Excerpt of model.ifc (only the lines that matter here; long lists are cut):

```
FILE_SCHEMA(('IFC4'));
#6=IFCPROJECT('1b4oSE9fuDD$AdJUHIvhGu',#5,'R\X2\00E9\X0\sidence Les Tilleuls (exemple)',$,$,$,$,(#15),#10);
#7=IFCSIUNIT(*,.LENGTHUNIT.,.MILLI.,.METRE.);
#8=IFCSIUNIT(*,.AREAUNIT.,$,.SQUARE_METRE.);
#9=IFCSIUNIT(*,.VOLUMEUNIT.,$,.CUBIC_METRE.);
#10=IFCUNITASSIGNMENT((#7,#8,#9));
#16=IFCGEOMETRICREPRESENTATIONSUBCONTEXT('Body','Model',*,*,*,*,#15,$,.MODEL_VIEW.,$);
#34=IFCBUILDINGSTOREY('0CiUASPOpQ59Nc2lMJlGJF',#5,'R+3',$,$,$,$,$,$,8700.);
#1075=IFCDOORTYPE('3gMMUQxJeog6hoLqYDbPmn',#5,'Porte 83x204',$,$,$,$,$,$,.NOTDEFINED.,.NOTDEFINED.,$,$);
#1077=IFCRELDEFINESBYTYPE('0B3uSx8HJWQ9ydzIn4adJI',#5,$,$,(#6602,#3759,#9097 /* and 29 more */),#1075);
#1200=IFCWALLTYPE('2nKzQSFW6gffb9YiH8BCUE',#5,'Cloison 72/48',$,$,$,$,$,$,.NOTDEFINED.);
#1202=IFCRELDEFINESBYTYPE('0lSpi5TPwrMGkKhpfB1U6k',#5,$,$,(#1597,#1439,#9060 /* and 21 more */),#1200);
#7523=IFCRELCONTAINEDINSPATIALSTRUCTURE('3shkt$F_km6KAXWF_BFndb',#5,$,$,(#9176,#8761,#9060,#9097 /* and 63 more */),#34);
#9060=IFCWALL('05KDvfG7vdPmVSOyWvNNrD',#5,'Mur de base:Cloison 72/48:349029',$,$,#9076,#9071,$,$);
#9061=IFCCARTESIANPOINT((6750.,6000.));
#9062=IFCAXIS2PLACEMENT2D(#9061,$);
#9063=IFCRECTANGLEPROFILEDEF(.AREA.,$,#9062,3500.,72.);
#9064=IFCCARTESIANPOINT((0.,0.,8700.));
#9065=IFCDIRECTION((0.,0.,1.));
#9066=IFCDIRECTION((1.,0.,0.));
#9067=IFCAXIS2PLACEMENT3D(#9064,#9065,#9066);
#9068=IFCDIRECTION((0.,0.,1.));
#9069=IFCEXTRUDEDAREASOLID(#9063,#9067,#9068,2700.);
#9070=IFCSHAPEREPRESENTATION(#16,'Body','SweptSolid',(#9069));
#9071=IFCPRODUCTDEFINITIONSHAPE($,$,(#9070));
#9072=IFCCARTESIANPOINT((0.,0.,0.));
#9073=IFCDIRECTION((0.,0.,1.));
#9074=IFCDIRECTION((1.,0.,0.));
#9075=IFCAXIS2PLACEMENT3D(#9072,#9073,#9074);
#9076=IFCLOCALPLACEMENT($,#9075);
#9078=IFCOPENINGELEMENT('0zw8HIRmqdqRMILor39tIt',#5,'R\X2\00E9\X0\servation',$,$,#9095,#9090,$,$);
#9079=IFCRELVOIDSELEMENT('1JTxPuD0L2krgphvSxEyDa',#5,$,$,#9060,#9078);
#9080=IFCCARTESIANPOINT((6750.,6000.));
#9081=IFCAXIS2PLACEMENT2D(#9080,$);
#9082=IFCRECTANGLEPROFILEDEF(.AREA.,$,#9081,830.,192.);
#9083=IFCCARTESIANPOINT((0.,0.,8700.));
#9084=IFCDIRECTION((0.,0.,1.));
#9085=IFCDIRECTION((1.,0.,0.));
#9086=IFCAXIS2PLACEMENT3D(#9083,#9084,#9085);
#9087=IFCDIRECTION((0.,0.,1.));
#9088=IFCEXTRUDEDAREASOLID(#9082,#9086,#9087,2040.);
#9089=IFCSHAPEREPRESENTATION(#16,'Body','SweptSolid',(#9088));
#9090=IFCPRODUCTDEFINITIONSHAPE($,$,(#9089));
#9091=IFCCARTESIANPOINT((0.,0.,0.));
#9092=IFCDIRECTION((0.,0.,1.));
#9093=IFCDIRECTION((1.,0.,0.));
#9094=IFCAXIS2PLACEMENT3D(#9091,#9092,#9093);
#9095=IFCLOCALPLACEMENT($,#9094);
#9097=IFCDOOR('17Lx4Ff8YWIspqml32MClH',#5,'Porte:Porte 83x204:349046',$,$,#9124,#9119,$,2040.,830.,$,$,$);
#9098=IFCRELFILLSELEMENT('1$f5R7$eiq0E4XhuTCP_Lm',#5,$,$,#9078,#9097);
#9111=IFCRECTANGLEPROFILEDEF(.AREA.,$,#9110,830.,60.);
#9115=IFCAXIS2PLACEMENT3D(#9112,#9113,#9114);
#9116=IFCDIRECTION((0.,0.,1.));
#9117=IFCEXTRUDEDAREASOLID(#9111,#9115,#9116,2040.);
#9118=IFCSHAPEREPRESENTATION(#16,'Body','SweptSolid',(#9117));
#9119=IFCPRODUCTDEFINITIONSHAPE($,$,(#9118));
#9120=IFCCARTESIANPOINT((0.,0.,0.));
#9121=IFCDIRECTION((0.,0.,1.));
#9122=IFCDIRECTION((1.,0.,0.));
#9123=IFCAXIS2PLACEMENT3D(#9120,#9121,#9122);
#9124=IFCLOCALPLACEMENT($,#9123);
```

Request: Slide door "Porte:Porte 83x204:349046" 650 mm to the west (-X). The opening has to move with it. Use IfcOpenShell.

```python
import ifcopenshell
import ifcopenshell.api.geometry
import ifcopenshell.util.placement
import ifcopenshell.util.unit

model = ifcopenshell.open("model.ifc")
unit_scale = ifcopenshell.util.unit.calculate_unit_scale(model)

door = model.by_guid("17Lx4Ff8YWIspqml32MClH")
opening = door.FillsVoids[0].RelatingOpeningElement
wall = opening.VoidsElements[0].RelatingBuildingElement

wall_matrix = ifcopenshell.util.placement.get_local_placement(wall.ObjectPlacement)
shift = wall_matrix[:3, 0] * -0.65 / unit_scale
before = ifcopenshell.util.placement.get_local_placement(door.ObjectPlacement)[:3, 3].copy()

# The door is not placed relative to its opening, so move both.
for product in (opening, door):
    matrix = ifcopenshell.util.placement.get_local_placement(product.ObjectPlacement)
    matrix[:3, 3] += shift
    ifcopenshell.api.geometry.edit_object_placement(model, product=product, matrix=matrix, is_si=False)

after = ifcopenshell.util.placement.get_local_placement(door.ObjectPlacement)[:3, 3]
print("door moved by", (after - before).round(3) + 0.0)

model.write("model-out.ifc")
```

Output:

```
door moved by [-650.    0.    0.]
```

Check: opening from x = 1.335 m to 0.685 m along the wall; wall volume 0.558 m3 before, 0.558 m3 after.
